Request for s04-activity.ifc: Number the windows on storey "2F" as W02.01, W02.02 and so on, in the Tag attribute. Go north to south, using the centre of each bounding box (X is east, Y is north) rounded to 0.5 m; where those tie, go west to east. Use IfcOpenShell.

First a look at what the model holds.

```python
import ifcopenshell
import ifcopenshell.util.element
import ifcopenshell.util.placement

model = ifcopenshell.open("s04-activity.ifc")
print(model.schema)
storey = next(s for s in model.by_type("IfcBuildingStorey") if s.Name == "2F")
windows = [e for e in ifcopenshell.util.element.get_decomposition(storey) if e.is_a("IfcWindow")]
for e in sorted(windows, key=lambda e: e.id()):
    origin = ifcopenshell.util.placement.get_local_placement(e.ObjectPlacement)[:3, 3]
    print(e.id(), e.Tag, e.Name, origin.round(2) + 0.0, sep=" | ")
```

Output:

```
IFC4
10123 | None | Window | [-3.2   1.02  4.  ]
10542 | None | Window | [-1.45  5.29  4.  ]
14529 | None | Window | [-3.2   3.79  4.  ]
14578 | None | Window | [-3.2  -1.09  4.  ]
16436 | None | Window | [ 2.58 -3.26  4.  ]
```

```python
import ifcopenshell
import ifcopenshell.geom
import ifcopenshell.util.element
import ifcopenshell.util.shape

model = ifcopenshell.open("s04-activity.ifc")
settings = ifcopenshell.geom.settings()
settings.set("use-world-coords", True)


def centre(element):
    shape = ifcopenshell.geom.create_shape(settings, element)
    return ifcopenshell.util.shape.get_bbox_centroid(shape.geometry)


storey = next(s for s in model.by_type("IfcBuildingStorey") if s.Name == "2F")
windows = [e for e in ifcopenshell.util.element.get_decomposition(storey) if e.is_a("IfcWindow")]

# Insertion points can sit at a corner or the storey origin, so sort by the geometry (in metres).
centres = {e: centre(e) for e in windows}
windows.sort(key=lambda e: (-round(centres[e][1] / 0.5), centres[e][0]))

for i, e in enumerate(windows, start=1):
    number = f"W02.{i:02d}"
    e.Tag = number
    print(e.id(), number)

model.write("s04-activity_rev.ifc")
```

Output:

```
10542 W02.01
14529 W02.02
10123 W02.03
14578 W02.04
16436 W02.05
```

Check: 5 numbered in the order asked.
